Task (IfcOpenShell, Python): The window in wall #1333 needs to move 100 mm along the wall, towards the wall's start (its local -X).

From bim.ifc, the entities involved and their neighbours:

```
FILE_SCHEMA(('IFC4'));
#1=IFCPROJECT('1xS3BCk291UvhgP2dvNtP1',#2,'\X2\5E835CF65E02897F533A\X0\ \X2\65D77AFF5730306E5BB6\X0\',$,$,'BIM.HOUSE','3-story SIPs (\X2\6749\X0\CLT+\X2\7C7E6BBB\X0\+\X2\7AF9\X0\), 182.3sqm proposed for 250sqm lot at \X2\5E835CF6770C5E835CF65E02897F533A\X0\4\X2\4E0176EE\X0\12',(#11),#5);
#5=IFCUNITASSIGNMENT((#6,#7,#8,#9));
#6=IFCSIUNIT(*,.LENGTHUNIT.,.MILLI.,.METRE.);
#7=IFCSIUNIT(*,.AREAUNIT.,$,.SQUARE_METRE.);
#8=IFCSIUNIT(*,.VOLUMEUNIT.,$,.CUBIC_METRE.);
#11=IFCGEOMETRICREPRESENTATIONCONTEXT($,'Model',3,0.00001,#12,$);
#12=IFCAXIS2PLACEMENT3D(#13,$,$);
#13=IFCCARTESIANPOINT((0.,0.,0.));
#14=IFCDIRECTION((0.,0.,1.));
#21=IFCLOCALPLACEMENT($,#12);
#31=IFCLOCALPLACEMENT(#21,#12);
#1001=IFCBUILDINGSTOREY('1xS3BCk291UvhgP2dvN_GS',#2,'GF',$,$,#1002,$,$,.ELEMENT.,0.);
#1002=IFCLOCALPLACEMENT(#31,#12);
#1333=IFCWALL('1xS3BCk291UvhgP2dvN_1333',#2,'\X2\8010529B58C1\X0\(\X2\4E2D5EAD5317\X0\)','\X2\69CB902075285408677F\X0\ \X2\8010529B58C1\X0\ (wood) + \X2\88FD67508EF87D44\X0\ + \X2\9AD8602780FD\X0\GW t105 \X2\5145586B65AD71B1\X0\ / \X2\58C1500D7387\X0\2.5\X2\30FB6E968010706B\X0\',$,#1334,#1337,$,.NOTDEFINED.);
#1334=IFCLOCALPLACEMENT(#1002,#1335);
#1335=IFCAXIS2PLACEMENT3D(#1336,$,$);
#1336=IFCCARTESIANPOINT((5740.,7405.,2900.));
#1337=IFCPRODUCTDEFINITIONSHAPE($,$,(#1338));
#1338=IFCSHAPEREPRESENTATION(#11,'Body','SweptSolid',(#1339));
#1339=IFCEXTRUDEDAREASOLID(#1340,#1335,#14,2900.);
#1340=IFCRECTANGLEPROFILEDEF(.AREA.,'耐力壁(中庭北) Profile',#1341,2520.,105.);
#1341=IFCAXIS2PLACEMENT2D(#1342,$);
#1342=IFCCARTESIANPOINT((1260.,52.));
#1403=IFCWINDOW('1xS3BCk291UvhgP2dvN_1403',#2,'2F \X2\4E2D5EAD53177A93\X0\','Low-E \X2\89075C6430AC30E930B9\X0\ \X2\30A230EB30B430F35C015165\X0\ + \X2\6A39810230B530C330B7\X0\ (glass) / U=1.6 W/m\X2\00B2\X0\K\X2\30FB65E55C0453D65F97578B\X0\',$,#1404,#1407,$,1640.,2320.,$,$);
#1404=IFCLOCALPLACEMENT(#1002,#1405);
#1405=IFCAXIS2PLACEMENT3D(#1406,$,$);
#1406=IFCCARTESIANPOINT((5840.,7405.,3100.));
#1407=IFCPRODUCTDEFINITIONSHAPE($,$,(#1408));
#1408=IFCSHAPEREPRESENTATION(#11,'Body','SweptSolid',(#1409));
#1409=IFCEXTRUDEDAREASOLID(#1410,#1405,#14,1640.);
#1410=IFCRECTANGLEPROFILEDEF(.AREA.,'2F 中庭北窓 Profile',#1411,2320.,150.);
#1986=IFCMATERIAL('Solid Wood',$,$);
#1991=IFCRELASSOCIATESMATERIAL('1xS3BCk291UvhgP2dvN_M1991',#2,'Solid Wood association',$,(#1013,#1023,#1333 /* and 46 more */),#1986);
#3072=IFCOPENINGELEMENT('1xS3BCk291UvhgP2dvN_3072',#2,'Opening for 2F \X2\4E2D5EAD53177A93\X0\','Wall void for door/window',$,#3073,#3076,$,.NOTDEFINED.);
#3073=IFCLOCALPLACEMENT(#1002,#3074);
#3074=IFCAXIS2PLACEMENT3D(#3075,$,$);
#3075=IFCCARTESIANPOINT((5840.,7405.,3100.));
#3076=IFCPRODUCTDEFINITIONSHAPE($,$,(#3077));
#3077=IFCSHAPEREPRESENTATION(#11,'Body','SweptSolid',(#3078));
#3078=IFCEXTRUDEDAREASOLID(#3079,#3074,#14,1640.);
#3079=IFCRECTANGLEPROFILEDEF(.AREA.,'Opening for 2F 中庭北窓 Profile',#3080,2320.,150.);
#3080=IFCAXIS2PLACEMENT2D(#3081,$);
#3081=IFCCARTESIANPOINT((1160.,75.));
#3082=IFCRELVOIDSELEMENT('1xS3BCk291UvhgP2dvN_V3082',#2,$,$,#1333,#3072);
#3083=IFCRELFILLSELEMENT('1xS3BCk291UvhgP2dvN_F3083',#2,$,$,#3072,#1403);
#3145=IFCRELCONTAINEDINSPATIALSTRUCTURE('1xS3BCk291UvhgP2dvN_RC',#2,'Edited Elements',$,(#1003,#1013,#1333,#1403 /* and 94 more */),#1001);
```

```python
import ifcopenshell
import ifcopenshell.api.geometry
import ifcopenshell.util.placement
import ifcopenshell.util.unit

model = ifcopenshell.open("bim.ifc")
unit_scale = ifcopenshell.util.unit.calculate_unit_scale(model)

window = model.by_id(1403)
opening = window.FillsVoids[0].RelatingOpeningElement
wall = opening.VoidsElements[0].RelatingBuildingElement

wall_matrix = ifcopenshell.util.placement.get_local_placement(wall.ObjectPlacement)
shift = wall_matrix[:3, 0] * -0.1 / unit_scale
before = ifcopenshell.util.placement.get_local_placement(window.ObjectPlacement)[:3, 3].copy()

# The window is not placed relative to its opening, so move both.
for product in (opening, window):
    matrix = ifcopenshell.util.placement.get_local_placement(product.ObjectPlacement)
    matrix[:3, 3] += shift
    ifcopenshell.api.geometry.edit_object_placement(model, product=product, matrix=matrix, is_si=False)

after = ifcopenshell.util.placement.get_local_placement(window.ObjectPlacement)[:3, 3]
print("window moved by", (after - before).round(3) + 0.0)

model.write("bim_v2.ifc")
```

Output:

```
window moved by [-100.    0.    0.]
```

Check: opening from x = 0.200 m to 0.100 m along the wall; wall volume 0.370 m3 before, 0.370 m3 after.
